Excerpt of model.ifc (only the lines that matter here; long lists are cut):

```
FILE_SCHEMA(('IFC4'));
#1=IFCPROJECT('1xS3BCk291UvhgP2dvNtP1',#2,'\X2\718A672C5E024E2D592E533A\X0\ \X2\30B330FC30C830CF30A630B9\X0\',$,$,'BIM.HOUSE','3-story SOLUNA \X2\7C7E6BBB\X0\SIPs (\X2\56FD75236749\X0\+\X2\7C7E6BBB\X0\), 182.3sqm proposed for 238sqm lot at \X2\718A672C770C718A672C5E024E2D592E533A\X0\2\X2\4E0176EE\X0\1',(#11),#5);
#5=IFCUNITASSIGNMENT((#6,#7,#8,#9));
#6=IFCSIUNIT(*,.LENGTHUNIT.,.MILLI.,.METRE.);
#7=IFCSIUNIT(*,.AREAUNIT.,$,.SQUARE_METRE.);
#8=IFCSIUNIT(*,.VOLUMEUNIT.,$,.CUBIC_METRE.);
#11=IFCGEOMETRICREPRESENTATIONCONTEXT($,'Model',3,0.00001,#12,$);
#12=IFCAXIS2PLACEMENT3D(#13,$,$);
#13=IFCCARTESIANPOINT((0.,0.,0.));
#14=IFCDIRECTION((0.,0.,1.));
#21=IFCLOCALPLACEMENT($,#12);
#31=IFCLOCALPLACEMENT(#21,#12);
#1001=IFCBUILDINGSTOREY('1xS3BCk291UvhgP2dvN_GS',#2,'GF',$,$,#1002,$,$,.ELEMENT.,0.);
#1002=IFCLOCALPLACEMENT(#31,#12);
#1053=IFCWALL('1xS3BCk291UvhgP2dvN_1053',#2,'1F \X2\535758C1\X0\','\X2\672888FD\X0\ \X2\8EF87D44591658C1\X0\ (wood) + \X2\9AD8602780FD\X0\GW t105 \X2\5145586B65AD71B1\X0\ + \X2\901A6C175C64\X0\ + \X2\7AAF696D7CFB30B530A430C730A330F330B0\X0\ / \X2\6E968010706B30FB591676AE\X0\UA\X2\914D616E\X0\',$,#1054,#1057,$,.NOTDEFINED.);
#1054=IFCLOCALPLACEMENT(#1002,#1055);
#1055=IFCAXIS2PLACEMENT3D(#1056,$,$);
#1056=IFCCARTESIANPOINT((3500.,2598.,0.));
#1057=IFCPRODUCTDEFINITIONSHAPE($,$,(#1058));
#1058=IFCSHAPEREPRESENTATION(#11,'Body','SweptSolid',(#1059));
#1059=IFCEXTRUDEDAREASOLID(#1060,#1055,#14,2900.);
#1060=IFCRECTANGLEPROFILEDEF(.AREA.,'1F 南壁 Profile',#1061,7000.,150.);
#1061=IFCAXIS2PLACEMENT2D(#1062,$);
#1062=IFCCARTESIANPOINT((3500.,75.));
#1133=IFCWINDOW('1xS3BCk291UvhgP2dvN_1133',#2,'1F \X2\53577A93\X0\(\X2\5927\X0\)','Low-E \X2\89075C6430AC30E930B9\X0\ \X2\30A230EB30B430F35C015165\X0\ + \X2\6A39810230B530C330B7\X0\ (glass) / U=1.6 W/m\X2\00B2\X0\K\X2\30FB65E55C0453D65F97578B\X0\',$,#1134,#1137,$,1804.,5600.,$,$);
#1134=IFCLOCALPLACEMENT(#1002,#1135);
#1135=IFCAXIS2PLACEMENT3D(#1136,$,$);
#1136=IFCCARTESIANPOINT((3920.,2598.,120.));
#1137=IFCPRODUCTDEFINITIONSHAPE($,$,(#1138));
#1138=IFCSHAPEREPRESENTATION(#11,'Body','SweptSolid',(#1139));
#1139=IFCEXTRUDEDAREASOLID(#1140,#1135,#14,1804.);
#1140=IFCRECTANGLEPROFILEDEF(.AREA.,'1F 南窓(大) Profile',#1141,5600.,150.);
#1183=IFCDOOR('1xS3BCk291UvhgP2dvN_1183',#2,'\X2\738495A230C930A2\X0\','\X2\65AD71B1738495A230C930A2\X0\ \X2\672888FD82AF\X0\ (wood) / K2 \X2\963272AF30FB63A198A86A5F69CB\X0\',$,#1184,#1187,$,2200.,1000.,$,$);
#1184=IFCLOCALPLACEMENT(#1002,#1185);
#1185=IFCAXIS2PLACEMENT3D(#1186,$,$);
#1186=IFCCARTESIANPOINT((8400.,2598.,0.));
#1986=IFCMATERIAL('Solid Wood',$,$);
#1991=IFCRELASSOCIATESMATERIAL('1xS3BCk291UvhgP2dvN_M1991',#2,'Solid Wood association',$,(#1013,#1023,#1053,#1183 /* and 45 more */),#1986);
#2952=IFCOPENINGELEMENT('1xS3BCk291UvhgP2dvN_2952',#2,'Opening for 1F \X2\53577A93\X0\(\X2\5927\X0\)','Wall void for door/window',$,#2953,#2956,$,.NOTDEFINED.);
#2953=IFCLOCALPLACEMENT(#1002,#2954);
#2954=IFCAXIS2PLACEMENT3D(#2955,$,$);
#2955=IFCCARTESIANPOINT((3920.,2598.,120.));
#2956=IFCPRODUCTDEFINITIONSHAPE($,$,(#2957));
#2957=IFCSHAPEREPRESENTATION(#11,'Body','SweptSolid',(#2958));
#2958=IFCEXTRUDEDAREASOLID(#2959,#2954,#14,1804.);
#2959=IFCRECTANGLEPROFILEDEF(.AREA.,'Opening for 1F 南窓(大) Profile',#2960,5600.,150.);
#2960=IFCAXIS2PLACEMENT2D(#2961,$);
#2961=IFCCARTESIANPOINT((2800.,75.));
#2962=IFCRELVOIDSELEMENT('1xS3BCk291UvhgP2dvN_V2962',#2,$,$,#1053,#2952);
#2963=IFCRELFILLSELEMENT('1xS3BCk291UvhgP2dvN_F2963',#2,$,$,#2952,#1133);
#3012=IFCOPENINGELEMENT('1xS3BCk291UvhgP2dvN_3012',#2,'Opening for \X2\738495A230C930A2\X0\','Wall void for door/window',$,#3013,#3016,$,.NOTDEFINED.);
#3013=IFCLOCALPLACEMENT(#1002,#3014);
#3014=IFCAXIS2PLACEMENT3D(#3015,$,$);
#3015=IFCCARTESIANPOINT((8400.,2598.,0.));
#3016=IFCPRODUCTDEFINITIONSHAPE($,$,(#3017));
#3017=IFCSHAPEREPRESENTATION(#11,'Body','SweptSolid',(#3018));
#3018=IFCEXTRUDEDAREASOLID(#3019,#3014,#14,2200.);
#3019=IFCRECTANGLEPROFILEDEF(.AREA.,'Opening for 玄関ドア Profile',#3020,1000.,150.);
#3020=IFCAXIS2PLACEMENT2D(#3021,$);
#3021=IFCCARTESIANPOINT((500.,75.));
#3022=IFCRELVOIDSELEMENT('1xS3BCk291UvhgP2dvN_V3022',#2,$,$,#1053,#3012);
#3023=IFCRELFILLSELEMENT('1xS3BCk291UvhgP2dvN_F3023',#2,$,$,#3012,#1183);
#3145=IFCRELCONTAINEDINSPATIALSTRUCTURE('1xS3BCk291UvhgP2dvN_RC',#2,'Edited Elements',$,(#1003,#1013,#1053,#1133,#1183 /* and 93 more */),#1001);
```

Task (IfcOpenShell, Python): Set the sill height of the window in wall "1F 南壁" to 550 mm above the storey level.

```python
import numpy as np
import ifcopenshell
import ifcopenshell.api.geometry
import ifcopenshell.geom
import ifcopenshell.util.element
import ifcopenshell.util.placement
import ifcopenshell.util.shape
import ifcopenshell.util.unit

model = ifcopenshell.open("model.ifc")
unit_scale = ifcopenshell.util.unit.calculate_unit_scale(model)

window = model.by_guid("1xS3BCk291UvhgP2dvN_1133")
opening = window.FillsVoids[0].RelatingOpeningElement
storey = ifcopenshell.util.element.get_container(window, ifc_class="IfcBuildingStorey")
level = ifcopenshell.util.placement.get_local_placement(storey.ObjectPlacement)[2, 3]

# The opening's origin need not be at the sill, so measure its lowest point.
shape = ifcopenshell.geom.create_shape(ifcopenshell.geom.settings(), opening)
bottom = ifcopenshell.util.shape.get_shape_bottom_elevation(shape, shape.geometry) / unit_scale
dz = level + 550.0 - bottom

shift = np.array([0.0, 0.0, dz])
# The window is not placed relative to its opening, so move both.
for product in (opening, window):
    matrix = ifcopenshell.util.placement.get_local_placement(product.ObjectPlacement)
    matrix[:3, 3] += shift
    ifcopenshell.api.geometry.edit_object_placement(model, product=product, matrix=matrix, is_si=False)

print(f"moved by {dz * unit_scale:+.3f} m")

model.write("model_updated.ifc")
```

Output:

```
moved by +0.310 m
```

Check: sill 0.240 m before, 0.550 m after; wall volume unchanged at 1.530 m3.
